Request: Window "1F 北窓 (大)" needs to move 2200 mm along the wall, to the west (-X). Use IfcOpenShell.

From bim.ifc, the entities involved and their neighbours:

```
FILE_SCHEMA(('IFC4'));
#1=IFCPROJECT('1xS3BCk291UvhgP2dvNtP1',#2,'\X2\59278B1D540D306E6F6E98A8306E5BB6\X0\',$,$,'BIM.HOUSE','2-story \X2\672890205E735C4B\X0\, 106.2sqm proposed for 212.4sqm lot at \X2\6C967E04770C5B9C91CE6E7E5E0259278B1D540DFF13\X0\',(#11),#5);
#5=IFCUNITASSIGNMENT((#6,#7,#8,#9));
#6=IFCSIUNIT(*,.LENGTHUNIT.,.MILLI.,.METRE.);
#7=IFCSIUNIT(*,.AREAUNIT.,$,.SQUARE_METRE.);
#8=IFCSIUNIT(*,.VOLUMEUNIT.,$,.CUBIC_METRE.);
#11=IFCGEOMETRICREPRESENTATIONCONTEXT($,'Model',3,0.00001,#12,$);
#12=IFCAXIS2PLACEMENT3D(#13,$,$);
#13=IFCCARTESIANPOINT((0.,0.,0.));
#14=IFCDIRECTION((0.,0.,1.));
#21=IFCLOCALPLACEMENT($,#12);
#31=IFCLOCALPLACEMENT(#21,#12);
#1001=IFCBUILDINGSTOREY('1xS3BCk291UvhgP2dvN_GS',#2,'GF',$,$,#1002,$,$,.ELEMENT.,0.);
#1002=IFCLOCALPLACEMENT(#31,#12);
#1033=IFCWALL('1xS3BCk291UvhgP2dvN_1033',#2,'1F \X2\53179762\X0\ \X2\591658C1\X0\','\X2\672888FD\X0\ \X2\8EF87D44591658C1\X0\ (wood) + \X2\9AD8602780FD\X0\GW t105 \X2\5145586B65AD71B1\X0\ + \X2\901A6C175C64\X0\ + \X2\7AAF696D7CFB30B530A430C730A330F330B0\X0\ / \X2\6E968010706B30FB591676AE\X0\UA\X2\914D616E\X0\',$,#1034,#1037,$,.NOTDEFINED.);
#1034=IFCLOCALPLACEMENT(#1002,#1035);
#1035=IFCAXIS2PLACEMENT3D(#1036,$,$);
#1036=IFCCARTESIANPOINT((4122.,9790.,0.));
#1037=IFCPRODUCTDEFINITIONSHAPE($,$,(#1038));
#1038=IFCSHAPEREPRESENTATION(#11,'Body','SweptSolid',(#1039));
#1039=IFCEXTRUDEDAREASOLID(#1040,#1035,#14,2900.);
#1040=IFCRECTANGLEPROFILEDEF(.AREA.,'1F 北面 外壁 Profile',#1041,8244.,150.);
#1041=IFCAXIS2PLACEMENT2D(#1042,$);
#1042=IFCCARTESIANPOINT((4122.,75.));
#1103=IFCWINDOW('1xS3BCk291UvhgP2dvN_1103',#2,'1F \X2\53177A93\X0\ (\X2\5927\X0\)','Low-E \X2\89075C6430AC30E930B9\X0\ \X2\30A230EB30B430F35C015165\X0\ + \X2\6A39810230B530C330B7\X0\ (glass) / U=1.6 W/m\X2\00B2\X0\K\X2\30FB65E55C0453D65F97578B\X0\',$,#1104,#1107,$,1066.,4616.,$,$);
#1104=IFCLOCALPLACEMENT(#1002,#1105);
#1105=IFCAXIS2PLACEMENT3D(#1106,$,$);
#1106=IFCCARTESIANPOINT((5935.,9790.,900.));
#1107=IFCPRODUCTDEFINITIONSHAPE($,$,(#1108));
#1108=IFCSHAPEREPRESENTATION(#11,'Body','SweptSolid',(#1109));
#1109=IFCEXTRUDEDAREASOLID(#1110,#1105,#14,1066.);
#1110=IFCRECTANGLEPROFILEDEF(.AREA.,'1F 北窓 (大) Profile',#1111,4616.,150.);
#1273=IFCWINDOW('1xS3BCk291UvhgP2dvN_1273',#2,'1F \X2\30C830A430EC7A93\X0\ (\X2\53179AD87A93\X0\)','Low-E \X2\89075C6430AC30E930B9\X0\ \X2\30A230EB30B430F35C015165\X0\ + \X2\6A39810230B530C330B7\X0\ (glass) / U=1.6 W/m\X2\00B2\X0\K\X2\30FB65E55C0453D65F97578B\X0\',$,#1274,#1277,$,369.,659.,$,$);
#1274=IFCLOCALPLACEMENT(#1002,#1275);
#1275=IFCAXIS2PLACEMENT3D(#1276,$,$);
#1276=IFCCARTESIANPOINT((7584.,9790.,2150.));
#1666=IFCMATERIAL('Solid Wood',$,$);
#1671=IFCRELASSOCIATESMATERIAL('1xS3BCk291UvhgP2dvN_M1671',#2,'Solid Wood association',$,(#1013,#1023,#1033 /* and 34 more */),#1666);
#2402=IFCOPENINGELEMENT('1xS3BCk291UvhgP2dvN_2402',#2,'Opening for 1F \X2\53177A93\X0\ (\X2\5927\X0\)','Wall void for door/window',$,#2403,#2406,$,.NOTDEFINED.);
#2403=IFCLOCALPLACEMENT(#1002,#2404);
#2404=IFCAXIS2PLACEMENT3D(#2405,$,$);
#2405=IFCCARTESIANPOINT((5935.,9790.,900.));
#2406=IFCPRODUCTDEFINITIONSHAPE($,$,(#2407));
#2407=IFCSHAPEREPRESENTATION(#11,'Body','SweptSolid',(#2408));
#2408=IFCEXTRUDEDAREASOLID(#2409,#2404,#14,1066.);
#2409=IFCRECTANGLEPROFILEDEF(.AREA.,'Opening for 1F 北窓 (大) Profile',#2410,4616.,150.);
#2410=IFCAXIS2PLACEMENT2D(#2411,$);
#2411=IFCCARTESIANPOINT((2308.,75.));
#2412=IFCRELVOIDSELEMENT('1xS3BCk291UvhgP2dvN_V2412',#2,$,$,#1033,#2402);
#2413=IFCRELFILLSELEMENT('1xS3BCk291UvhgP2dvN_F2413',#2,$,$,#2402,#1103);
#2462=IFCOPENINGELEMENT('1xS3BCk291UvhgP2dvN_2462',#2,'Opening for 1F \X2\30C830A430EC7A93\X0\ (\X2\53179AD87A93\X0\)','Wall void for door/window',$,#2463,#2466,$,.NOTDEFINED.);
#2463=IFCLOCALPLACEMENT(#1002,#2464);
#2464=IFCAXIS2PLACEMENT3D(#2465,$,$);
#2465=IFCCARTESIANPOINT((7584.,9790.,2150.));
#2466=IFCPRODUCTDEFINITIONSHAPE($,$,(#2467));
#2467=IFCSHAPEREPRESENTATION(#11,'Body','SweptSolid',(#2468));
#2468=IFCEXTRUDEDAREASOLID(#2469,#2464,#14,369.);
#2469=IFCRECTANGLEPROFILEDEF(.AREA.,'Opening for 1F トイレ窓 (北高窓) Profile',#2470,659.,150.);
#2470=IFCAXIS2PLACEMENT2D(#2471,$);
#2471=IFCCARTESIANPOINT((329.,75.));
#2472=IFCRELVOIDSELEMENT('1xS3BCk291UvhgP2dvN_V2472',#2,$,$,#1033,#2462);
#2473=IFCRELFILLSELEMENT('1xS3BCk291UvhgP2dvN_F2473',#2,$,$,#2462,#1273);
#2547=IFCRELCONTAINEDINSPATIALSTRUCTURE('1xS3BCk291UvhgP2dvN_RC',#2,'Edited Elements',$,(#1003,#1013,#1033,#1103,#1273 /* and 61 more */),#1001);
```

```python
import ifcopenshell
import ifcopenshell.api.geometry
import ifcopenshell.util.placement
import ifcopenshell.util.unit

model = ifcopenshell.open("bim.ifc")
unit_scale = ifcopenshell.util.unit.calculate_unit_scale(model)

window = model.by_guid("1xS3BCk291UvhgP2dvN_1103")
opening = window.FillsVoids[0].RelatingOpeningElement
wall = opening.VoidsElements[0].RelatingBuildingElement

wall_matrix = ifcopenshell.util.placement.get_local_placement(wall.ObjectPlacement)
shift = wall_matrix[:3, 0] * -2.2 / unit_scale
before = ifcopenshell.util.placement.get_local_placement(window.ObjectPlacement)[:3, 3].copy()

# The window is not placed relative to its opening, so move both.
for product in (opening, window):
    matrix = ifcopenshell.util.placement.get_local_placement(product.ObjectPlacement)
    matrix[:3, 3] += shift
    ifcopenshell.api.geometry.edit_object_placement(model, product=product, matrix=matrix, is_si=False)

after = ifcopenshell.util.placement.get_local_placement(window.ObjectPlacement)[:3, 3]
print("window moved by", (after - before).round(3) + 0.0)

model.write("bim_v2.ifc")
```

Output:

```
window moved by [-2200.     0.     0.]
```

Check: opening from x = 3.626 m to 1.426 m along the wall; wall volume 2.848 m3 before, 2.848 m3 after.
